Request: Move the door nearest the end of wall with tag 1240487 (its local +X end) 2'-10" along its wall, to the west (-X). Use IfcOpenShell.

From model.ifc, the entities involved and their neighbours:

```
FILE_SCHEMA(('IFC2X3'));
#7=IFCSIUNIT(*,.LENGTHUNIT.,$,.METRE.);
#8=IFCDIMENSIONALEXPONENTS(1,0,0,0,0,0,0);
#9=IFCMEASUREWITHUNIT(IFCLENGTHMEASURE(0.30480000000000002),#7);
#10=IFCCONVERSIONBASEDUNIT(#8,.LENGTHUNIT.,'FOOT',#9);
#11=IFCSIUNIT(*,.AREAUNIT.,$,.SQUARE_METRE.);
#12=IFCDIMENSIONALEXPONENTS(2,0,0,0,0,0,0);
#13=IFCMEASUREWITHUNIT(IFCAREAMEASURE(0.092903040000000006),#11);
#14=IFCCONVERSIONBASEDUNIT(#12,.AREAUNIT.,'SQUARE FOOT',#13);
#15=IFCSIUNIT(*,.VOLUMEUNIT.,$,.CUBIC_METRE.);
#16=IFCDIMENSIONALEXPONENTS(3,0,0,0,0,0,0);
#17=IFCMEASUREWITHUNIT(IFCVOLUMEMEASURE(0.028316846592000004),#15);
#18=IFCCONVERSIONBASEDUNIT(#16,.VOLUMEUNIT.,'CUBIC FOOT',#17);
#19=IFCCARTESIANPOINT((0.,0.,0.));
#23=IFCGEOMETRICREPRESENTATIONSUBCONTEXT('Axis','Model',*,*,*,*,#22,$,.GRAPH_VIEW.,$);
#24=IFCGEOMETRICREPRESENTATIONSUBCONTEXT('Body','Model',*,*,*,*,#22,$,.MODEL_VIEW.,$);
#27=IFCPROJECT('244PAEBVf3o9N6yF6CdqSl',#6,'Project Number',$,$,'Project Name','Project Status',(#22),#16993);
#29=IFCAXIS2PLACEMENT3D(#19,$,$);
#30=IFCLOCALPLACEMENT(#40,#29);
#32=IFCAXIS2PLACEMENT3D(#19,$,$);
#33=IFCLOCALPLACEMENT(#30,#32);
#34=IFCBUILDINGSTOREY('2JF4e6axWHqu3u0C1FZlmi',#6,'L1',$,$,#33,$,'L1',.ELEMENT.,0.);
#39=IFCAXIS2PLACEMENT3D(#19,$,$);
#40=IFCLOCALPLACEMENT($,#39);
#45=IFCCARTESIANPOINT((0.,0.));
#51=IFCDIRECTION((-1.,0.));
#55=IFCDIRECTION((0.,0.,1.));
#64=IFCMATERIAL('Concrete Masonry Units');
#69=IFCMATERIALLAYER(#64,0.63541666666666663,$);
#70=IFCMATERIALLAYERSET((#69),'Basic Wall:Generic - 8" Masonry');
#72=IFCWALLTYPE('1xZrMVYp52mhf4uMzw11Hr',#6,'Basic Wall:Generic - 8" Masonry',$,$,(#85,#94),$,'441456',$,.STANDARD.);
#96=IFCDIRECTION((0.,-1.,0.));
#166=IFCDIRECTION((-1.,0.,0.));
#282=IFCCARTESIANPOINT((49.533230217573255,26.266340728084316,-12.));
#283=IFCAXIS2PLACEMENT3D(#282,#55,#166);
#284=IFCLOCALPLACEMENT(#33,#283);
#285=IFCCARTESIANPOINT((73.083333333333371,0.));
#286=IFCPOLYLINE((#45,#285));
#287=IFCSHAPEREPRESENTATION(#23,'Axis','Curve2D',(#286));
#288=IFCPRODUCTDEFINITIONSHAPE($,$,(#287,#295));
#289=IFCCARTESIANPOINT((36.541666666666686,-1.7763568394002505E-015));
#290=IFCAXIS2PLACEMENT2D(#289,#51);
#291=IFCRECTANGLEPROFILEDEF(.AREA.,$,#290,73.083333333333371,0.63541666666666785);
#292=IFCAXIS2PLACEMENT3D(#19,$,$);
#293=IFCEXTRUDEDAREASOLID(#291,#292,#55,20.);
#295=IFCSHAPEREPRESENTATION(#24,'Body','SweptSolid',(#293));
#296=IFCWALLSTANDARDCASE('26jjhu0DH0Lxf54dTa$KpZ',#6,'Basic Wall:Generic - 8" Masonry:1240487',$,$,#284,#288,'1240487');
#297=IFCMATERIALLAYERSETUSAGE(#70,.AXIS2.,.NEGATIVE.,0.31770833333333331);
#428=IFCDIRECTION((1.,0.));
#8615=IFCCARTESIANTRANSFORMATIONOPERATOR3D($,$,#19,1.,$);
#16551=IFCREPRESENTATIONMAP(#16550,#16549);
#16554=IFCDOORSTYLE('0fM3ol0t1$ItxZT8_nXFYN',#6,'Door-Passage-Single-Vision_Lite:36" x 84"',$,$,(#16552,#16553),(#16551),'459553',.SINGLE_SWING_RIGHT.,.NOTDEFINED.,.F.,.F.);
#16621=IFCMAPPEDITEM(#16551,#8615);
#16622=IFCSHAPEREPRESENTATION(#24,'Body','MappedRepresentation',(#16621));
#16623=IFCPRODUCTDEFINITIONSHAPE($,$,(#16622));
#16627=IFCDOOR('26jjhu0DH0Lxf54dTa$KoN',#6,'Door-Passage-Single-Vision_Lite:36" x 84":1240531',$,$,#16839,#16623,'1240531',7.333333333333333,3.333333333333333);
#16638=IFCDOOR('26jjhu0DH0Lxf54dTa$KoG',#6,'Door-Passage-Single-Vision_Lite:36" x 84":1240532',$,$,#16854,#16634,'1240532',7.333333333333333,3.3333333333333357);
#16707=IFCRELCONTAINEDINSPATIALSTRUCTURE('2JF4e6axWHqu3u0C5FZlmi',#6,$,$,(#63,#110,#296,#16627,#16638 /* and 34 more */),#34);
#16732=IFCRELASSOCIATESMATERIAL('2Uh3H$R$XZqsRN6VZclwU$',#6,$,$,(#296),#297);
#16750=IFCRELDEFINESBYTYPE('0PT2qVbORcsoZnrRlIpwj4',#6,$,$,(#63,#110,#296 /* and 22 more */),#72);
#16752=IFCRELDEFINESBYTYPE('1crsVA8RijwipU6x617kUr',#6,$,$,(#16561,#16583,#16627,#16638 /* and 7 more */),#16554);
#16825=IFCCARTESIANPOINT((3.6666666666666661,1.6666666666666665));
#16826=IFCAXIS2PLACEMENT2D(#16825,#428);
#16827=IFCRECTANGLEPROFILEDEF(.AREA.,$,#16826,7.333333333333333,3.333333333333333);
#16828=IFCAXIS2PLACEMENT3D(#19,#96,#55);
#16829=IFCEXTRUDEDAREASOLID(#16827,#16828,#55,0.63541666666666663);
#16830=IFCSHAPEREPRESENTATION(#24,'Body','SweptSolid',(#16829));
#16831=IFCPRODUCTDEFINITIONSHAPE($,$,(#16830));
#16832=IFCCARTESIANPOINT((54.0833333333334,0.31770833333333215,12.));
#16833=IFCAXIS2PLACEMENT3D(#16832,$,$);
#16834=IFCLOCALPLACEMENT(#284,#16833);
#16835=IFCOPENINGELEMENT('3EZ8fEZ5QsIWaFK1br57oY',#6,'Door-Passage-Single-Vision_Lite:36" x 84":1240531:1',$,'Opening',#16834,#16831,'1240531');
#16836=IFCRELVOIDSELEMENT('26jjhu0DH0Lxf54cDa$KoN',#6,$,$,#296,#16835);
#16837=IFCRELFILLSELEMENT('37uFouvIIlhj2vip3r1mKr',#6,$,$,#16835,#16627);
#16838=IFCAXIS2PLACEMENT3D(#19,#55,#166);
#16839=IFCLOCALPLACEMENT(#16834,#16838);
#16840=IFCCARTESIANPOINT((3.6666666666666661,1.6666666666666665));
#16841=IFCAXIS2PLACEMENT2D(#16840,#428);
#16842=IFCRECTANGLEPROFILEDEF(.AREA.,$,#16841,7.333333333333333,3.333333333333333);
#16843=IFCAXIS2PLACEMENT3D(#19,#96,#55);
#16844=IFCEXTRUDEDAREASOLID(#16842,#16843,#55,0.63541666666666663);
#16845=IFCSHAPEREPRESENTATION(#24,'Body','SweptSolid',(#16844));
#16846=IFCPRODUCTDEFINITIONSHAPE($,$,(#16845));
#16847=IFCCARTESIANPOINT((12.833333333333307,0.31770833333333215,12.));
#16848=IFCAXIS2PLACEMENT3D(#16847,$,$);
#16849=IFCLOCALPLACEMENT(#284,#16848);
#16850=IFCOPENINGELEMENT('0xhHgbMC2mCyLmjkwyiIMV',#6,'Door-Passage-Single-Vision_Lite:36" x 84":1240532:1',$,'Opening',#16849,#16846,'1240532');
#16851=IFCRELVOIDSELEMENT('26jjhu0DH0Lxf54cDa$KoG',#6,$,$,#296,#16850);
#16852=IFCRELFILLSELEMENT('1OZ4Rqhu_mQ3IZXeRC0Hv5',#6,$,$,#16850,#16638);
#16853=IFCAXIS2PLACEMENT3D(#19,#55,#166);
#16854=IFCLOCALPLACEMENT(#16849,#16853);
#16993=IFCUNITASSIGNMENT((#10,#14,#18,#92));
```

```python
import ifcopenshell
import ifcopenshell.api.geometry
import ifcopenshell.util.placement
import ifcopenshell.util.unit

model = ifcopenshell.open("model.ifc")
unit_scale = ifcopenshell.util.unit.calculate_unit_scale(model)

door = model.by_id(16627)
opening = door.FillsVoids[0].RelatingOpeningElement
wall = opening.VoidsElements[0].RelatingBuildingElement

wall_matrix = ifcopenshell.util.placement.get_local_placement(wall.ObjectPlacement)
shift = wall_matrix[:3, 0] * 34 * 0.0254 / unit_scale
before = ifcopenshell.util.placement.get_local_placement(door.ObjectPlacement)[:3, 3].copy()

# The door is placed relative to its opening, so it follows when the opening moves.
matrix = ifcopenshell.util.placement.get_local_placement(opening.ObjectPlacement)
matrix[:3, 3] += shift
ifcopenshell.api.geometry.edit_object_placement(
    model, product=opening, matrix=matrix, is_si=False, should_transform_children=True
)

after = ifcopenshell.util.placement.get_local_placement(door.ObjectPlacement)[:3, 3]
print("door moved by", (after - before).round(3) + 0.0)

model.write("model-out.ifc")
```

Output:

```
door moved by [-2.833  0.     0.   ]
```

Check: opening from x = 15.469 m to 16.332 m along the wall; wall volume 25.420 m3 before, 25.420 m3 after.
